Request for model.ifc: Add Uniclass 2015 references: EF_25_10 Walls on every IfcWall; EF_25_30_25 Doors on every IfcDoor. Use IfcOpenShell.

First a look at what the model holds.

```python
import ifcopenshell

model = ifcopenshell.open("model.ifc")
print(model.schema)
print("classifications:", [c.Name for c in model.by_type("IfcClassification")])
for ifc_class in ("IfcDoor", "IfcRoof", "IfcStair", "IfcWall", "IfcWindow"):
    print(ifc_class, len(model.by_type(ifc_class)))
```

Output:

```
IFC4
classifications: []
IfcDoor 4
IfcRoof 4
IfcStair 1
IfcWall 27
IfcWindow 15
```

```python
import ifcopenshell
import ifcopenshell.api.classification

model = ifcopenshell.open("model.ifc")

system = ifcopenshell.api.classification.add_classification(model, classification="Uniclass 2015")

codes = {
    "IfcWall": ("EF_25_10", "Walls"),
    "IfcDoor": ("EF_25_30_25", "Doors"),
}
for ifc_class, (code, name) in codes.items():
    products = model.by_type(ifc_class)
    ifcopenshell.api.classification.add_reference(
        model, products=products, classification=system, identification=code, name=name
    )
    print(code, len(products))

model.write("model_rev.ifc")
```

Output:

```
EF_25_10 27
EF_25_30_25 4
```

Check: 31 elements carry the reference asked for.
